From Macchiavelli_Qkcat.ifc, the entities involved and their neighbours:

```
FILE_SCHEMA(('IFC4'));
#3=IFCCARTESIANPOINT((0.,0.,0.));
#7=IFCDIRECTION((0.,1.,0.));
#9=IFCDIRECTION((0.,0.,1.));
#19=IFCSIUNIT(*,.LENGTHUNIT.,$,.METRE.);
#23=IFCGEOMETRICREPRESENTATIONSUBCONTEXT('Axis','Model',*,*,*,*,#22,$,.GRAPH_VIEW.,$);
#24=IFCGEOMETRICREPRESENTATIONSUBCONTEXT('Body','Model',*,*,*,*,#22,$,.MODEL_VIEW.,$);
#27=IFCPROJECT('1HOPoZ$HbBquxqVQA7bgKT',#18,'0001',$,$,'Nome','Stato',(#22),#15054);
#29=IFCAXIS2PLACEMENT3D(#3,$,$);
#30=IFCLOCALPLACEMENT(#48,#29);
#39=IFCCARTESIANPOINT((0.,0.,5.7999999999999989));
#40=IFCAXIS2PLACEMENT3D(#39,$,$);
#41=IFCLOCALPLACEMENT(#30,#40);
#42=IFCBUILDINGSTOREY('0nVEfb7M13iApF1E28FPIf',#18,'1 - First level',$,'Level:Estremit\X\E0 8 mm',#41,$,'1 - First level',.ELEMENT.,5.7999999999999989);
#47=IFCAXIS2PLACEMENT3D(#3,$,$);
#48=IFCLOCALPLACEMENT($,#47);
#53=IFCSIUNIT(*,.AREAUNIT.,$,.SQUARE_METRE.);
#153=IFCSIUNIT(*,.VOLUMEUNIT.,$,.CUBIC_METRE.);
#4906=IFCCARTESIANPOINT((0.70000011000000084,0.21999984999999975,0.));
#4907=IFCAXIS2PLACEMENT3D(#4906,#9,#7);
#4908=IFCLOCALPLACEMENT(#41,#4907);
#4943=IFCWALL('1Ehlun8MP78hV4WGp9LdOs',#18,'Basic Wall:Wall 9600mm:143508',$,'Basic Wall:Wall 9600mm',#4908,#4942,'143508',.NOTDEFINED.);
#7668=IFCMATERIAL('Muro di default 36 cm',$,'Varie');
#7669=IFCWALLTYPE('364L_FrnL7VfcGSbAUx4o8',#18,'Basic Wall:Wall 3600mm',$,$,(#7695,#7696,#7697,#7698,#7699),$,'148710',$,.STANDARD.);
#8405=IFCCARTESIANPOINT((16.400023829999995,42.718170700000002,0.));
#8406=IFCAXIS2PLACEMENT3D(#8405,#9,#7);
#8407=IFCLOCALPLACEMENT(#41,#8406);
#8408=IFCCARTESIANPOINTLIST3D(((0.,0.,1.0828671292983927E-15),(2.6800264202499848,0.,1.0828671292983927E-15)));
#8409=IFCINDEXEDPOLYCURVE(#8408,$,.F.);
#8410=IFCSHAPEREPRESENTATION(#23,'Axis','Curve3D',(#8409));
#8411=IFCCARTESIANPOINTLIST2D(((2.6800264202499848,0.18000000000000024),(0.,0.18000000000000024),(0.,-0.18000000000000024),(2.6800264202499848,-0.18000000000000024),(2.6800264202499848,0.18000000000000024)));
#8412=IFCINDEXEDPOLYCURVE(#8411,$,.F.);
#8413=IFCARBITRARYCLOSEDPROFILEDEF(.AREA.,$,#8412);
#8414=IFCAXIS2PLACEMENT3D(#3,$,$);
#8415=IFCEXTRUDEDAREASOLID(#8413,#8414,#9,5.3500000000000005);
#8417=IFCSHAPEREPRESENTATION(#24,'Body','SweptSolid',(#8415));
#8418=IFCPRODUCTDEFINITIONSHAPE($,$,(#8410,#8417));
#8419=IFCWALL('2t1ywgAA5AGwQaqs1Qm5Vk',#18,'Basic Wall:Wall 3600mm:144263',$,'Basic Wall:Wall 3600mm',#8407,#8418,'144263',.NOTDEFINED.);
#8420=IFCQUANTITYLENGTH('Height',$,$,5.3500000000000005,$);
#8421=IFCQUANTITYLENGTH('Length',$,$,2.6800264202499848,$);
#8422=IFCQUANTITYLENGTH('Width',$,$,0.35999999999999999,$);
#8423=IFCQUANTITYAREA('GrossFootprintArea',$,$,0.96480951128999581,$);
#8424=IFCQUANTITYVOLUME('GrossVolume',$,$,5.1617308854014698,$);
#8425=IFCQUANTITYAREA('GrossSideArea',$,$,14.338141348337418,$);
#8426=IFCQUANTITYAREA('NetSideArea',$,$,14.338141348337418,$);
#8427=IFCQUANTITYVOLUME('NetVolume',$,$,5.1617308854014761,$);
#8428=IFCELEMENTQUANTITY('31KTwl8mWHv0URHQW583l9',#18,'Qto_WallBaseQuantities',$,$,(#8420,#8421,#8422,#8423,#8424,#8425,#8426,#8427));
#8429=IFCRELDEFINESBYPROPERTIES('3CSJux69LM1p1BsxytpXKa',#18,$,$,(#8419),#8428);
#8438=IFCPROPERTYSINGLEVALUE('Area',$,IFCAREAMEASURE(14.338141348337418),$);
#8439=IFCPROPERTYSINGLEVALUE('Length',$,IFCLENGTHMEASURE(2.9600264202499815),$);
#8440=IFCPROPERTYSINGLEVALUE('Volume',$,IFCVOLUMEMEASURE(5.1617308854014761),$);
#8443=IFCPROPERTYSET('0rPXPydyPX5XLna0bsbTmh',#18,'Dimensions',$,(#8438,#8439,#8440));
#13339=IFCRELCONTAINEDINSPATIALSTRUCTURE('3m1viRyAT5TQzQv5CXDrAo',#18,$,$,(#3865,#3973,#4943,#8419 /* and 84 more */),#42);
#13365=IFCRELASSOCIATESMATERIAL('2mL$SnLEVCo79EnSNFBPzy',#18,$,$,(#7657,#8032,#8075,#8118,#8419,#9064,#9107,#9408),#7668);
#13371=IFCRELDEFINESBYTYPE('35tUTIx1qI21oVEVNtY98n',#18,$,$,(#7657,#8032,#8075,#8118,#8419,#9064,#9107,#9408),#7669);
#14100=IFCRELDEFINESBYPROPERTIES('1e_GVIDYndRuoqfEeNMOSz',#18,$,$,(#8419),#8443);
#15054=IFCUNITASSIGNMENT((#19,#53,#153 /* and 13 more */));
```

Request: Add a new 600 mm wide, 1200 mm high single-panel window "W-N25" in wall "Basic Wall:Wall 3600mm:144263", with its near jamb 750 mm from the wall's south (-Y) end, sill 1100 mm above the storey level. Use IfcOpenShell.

```python
import numpy as np
import ifcopenshell
import ifcopenshell.api.feature
import ifcopenshell.api.geometry
import ifcopenshell.api.pset
import ifcopenshell.api.root
import ifcopenshell.api.spatial
import ifcopenshell.geom
import ifcopenshell.util.element
import ifcopenshell.util.placement
import ifcopenshell.util.representation
import ifcopenshell.util.shape
import ifcopenshell.util.unit

model = ifcopenshell.open("Macchiavelli_Qkcat.ifc")
unit_scale = ifcopenshell.util.unit.calculate_unit_scale(model)
area_scale = ifcopenshell.util.unit.calculate_unit_scale(model, "AREAUNIT")
volume_scale = ifcopenshell.util.unit.calculate_unit_scale(model, "VOLUMEUNIT")
settings = ifcopenshell.geom.settings()


def volume(element):
    """Net volume in cubic metres, openings subtracted."""
    shape = ifcopenshell.geom.create_shape(settings, element)
    return ifcopenshell.util.shape.get_volume(shape.geometry)


wall = model.by_id(8419)
storey = ifcopenshell.util.element.get_container(wall, ifc_class="IfcBuildingStorey")
context = ifcopenshell.util.representation.get_context(model, "Model", "Body", "MODEL_VIEW")
before = volume(wall)

width, height, from_end, sill = 0.6, 1.2, 0.75, 1.1  # metres

# The wall runs along its own X axis, and the end named is its -X end.
wall_shape = ifcopenshell.geom.create_shape(settings, wall)
x, y, z = ifcopenshell.util.shape.get_vertices(wall_shape.geometry).T
start = x.min() + from_end
face, thickness = float(y.min()), float(y.max() - y.min())
wall_matrix = ifcopenshell.util.placement.get_local_placement(wall.ObjectPlacement)
level = ifcopenshell.util.placement.get_local_placement(storey.ObjectPlacement)[2, 3]


def in_wall(x, y):
    """Placement at x, y metres in the wall's axes, at sill height."""
    matrix = wall_matrix.copy()
    matrix[:, 3] = wall_matrix @ np.array([x / unit_scale, y / unit_scale, 0.0, 1.0])
    matrix[2, 3] = level + sill / unit_scale
    return matrix


# Opening: a box that overshoots both wall faces by 50 mm.
opening = ifcopenshell.api.root.create_entity(model, ifc_class="IfcOpeningElement", predefined_type="OPENING")
box = ifcopenshell.api.geometry.add_wall_representation(
    model, context=context, length=width, height=height, thickness=thickness + 0.1
)
ifcopenshell.api.geometry.assign_representation(model, product=opening, representation=box)
ifcopenshell.api.geometry.edit_object_placement(model, product=opening, matrix=in_wall(start, face - 0.05), is_si=False)
ifcopenshell.api.feature.add_feature(model, feature=opening, element=wall)

window = ifcopenshell.api.root.create_entity(model, ifc_class="IfcWindow", name="W-N25", predefined_type="WINDOW")
window.OverallWidth, window.OverallHeight = width / unit_scale, height / unit_scale
window.PartitioningType = "SINGLE_PANEL"
body = ifcopenshell.api.geometry.add_window_representation(
    model,
    context=context,
    overall_width=window.OverallWidth,
    overall_height=window.OverallHeight,
    partition_type="SINGLE_PANEL",
)
ifcopenshell.api.geometry.assign_representation(model, product=window, representation=body)
ifcopenshell.api.spatial.assign_container(model, products=[window], relating_structure=storey)
ifcopenshell.api.feature.add_filling(model, opening=opening, element=window)

# Centre the window in the wall's thickness.
ifcopenshell.api.geometry.edit_object_placement(model, product=window, matrix=in_wall(start, face), is_si=False)
window_shape = ifcopenshell.geom.create_shape(settings, window)
depth = ifcopenshell.util.shape.get_vertices(window_shape.geometry)[:, 1]
offset = face + thickness / 2 - (depth.min() + depth.max()) / 2
ifcopenshell.api.geometry.edit_object_placement(model, product=window, matrix=in_wall(start, offset), is_si=False)

after = volume(wall)

# Update the wall's stored quantities.
qto = model.by_id(ifcopenshell.util.element.get_pset(wall, "Qto_WallBaseQuantities", should_inherit=False)["id"])
ifcopenshell.api.pset.edit_qto(model, qto=qto, properties={
    "NetSideArea": after / thickness / area_scale,
    "NetVolume": after / volume_scale,
})
pset = model.by_id(ifcopenshell.util.element.get_pset(wall, "Dimensions", should_inherit=False)["id"])
ifcopenshell.api.pset.edit_pset(model, pset=pset, properties={
    "Area": model.create_entity("IfcAreaMeasure", after / thickness / area_scale),
    "Volume": model.create_entity("IfcVolumeMeasure", after / volume_scale),
})

print(f"wall volume {before:.3f} -> {after:.3f} m3")

model.write("Macchiavelli_Qkcat_rev.ifc")
```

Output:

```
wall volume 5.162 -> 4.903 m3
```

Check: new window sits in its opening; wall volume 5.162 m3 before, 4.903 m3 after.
